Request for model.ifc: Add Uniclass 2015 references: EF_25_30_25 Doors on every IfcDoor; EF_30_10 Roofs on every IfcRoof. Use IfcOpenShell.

First a look at what the model holds.

```python
import ifcopenshell

model = ifcopenshell.open("model.ifc")
print(model.schema)
print("classifications:", [c.Name for c in model.by_type("IfcClassification")])
for ifc_class in ("IfcDoor", "IfcRoof", "IfcStair", "IfcWall", "IfcWindow"):
    print(ifc_class, len(model.by_type(ifc_class)))
```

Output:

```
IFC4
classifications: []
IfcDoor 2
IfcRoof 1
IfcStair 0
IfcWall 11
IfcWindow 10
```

```python
import ifcopenshell
import ifcopenshell.api.classification

model = ifcopenshell.open("model.ifc")

system = ifcopenshell.api.classification.add_classification(model, classification="Uniclass 2015")

codes = {
    "IfcDoor": ("EF_25_30_25", "Doors"),
    "IfcRoof": ("EF_30_10", "Roofs"),
}
for ifc_class, (code, name) in codes.items():
    products = model.by_type(ifc_class)
    ifcopenshell.api.classification.add_reference(
        model, products=products, classification=system, identification=code, name=name
    )
    print(code, len(products))

model.write("model-out.ifc")
```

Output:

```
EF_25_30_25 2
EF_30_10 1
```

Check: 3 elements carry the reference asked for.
